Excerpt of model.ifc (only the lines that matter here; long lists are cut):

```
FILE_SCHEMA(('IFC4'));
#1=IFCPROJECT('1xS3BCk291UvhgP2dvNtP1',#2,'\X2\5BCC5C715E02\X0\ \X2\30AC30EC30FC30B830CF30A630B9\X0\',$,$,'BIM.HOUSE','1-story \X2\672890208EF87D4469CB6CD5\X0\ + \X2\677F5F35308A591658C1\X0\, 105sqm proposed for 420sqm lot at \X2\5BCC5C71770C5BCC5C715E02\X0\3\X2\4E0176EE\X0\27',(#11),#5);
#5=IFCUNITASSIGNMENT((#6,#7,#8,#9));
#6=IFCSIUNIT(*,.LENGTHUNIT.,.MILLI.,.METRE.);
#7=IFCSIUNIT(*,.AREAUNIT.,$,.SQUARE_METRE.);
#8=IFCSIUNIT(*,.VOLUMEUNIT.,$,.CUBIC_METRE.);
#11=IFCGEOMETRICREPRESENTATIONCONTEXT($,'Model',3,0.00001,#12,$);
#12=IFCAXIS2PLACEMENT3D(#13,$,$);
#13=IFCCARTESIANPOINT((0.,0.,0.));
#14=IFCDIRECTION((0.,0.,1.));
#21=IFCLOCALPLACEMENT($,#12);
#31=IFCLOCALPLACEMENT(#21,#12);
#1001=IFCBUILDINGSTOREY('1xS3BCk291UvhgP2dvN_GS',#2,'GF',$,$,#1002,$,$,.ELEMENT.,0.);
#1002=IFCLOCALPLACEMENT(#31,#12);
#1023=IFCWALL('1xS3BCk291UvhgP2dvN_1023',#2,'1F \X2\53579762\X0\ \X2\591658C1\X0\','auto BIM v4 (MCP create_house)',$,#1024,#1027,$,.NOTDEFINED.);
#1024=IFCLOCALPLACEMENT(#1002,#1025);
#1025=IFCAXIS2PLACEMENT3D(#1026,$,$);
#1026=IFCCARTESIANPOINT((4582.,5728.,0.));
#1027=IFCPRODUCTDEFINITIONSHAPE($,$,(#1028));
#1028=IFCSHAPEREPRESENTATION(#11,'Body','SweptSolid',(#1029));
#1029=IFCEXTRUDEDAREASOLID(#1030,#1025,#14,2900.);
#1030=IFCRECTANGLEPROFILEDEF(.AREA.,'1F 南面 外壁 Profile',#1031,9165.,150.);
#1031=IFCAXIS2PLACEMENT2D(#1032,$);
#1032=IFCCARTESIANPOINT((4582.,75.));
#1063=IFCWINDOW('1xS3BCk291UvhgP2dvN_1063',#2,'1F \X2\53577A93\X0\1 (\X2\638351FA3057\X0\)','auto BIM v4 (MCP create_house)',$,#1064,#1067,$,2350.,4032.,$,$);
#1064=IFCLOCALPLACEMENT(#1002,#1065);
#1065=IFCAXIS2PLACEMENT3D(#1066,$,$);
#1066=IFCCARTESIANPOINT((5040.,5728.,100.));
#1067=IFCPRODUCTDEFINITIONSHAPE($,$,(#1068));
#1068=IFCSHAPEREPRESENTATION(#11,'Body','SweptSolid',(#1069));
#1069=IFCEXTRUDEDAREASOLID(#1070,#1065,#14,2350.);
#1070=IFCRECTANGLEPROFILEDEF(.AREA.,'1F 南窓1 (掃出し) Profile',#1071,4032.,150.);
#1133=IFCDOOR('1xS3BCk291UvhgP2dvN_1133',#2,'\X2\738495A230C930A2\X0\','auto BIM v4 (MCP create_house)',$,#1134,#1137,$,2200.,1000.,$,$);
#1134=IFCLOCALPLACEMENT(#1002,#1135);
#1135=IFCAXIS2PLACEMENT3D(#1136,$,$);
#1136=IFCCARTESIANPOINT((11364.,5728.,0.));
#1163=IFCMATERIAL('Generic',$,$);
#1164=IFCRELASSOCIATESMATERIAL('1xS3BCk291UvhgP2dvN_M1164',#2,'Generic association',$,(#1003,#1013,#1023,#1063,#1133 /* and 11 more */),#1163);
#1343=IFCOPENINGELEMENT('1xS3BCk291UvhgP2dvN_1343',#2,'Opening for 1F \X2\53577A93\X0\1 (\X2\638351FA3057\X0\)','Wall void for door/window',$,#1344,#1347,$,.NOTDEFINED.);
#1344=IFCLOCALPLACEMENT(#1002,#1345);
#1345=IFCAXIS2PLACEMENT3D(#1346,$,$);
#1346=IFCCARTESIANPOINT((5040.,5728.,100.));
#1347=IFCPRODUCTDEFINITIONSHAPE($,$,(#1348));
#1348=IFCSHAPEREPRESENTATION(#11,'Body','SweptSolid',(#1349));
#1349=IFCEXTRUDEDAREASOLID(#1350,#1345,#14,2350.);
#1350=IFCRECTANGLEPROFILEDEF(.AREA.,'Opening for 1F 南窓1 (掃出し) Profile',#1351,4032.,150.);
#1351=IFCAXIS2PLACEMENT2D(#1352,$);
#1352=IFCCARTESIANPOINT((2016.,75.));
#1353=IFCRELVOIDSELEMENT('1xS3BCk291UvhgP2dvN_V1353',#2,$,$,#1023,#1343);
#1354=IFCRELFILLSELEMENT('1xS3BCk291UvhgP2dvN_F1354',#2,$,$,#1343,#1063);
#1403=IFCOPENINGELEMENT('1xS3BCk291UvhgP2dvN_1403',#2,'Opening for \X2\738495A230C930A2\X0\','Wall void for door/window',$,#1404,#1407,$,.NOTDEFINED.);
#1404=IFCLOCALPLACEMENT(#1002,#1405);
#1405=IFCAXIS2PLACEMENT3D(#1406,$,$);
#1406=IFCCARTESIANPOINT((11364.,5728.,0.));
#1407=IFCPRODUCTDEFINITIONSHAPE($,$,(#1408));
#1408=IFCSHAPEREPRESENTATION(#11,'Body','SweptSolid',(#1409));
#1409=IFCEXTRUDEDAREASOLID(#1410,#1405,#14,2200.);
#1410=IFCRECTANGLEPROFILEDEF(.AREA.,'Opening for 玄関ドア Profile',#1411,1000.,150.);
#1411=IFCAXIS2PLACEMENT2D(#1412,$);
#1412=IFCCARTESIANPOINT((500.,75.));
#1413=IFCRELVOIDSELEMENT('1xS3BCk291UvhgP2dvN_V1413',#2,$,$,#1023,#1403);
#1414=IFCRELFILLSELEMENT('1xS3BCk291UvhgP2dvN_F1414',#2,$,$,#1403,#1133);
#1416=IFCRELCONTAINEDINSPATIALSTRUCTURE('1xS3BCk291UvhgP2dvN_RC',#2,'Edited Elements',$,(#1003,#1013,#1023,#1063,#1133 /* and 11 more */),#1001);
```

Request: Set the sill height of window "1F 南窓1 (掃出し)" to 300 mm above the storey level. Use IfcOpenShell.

```python
import numpy as np
import ifcopenshell
import ifcopenshell.api.geometry
import ifcopenshell.geom
import ifcopenshell.util.element
import ifcopenshell.util.placement
import ifcopenshell.util.shape
import ifcopenshell.util.unit

model = ifcopenshell.open("model.ifc")
unit_scale = ifcopenshell.util.unit.calculate_unit_scale(model)

window = model.by_id(1063)
opening = window.FillsVoids[0].RelatingOpeningElement
storey = ifcopenshell.util.element.get_container(window, ifc_class="IfcBuildingStorey")
level = ifcopenshell.util.placement.get_local_placement(storey.ObjectPlacement)[2, 3]

# The opening's origin need not be at the sill, so measure its lowest point.
shape = ifcopenshell.geom.create_shape(ifcopenshell.geom.settings(), opening)
bottom = ifcopenshell.util.shape.get_shape_bottom_elevation(shape, shape.geometry) / unit_scale
dz = level + 0.3 / unit_scale - bottom

shift = np.array([0.0, 0.0, dz])
# The window is not placed relative to its opening, so move both.
for product in (opening, window):
    matrix = ifcopenshell.util.placement.get_local_placement(product.ObjectPlacement)
    matrix[:3, 3] += shift
    ifcopenshell.api.geometry.edit_object_placement(model, product=product, matrix=matrix, is_si=False)

print(f"moved by {dz * unit_scale:+.3f} m")

model.write("model-out.ifc")
```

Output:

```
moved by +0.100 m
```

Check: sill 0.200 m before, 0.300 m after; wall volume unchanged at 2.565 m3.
